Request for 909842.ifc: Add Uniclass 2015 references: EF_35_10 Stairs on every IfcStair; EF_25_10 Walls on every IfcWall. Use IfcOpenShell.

First a look at what the model holds.

```python
import ifcopenshell

model = ifcopenshell.open("909842.ifc")
print(model.schema)
print("classifications:", [c.Name for c in model.by_type("IfcClassification")])
for ifc_class in ("IfcDoor", "IfcRoof", "IfcStair", "IfcWall", "IfcWindow"):
    print(ifc_class, len(model.by_type(ifc_class)))
```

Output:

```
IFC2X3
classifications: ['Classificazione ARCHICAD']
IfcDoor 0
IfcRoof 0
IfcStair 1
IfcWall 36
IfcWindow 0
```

```python
import ifcopenshell
import ifcopenshell.api.classification

model = ifcopenshell.open("909842.ifc")

# IFC2X3 requires Source and Edition and has no link from the project to the system.
system = model.create_entity("IfcClassification", Source="NBS", Edition="2015", Name="Uniclass 2015")

codes = {
    "IfcStair": ("EF_35_10", "Stairs"),
    "IfcWall": ("EF_25_10", "Walls"),
}
for ifc_class, (code, name) in codes.items():
    products = model.by_type(ifc_class)
    ifcopenshell.api.classification.add_reference(
        model, products=products, classification=system, identification=code, name=name
    )
    print(code, len(products))

model.write("909842-out.ifc")
```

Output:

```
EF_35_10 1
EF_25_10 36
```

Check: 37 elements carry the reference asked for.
